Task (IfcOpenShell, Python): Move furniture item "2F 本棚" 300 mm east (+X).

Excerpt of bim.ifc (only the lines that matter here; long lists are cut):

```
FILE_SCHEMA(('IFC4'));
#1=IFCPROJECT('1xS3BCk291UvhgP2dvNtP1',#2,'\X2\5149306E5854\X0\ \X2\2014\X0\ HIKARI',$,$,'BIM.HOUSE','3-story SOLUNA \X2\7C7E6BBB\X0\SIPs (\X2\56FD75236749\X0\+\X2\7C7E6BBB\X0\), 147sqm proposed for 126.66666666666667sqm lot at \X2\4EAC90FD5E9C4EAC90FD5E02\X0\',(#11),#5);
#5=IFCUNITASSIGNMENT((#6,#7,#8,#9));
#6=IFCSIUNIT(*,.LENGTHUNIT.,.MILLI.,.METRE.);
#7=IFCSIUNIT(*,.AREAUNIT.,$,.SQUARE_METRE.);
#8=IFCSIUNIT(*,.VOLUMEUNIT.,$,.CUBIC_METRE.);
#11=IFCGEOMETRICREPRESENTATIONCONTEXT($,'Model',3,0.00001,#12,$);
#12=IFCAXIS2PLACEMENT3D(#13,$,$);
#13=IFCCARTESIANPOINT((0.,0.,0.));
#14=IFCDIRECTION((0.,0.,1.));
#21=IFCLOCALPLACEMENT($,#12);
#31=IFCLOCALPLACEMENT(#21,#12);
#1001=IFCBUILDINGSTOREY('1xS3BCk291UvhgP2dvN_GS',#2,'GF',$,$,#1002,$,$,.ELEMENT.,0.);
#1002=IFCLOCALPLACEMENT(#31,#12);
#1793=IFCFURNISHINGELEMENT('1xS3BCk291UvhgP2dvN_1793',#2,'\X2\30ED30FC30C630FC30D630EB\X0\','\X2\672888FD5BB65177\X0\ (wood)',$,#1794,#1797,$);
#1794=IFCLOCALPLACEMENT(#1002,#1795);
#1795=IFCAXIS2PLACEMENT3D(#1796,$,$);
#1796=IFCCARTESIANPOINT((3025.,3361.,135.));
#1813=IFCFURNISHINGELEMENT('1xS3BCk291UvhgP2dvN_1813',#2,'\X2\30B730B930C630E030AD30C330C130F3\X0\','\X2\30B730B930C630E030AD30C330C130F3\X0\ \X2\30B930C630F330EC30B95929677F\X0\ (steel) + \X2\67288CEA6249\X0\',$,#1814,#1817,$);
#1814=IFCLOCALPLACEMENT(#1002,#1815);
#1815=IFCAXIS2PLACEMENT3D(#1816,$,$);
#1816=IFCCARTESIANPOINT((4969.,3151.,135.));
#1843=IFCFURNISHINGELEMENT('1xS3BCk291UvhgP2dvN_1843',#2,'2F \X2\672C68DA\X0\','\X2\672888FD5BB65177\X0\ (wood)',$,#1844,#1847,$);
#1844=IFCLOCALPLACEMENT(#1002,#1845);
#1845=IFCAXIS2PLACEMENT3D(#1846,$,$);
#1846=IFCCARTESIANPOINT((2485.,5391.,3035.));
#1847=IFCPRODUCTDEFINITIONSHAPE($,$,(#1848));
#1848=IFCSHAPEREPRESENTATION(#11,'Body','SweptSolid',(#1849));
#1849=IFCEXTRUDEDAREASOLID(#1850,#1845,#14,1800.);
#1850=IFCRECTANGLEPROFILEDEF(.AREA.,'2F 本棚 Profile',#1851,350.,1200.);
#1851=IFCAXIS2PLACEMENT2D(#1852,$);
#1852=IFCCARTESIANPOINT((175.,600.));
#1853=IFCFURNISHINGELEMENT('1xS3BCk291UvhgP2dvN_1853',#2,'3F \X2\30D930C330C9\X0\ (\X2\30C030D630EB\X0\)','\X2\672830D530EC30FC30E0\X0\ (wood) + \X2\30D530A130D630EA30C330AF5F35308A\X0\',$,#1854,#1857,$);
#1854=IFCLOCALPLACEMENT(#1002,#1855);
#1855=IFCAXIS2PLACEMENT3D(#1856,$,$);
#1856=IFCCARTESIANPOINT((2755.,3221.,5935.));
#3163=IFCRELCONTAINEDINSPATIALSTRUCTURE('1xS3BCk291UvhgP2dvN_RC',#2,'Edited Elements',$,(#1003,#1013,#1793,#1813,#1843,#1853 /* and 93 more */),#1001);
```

```python
import ifcopenshell
import ifcopenshell.api.geometry
import ifcopenshell.util.placement
import ifcopenshell.util.unit

model = ifcopenshell.open("bim.ifc")
unit_scale = ifcopenshell.util.unit.calculate_unit_scale(model)

item = model.by_guid("1xS3BCk291UvhgP2dvN_1843")
matrix = ifcopenshell.util.placement.get_local_placement(item.ObjectPlacement)
matrix[0, 3] += 0.3 / unit_scale
ifcopenshell.api.geometry.edit_object_placement(model, product=item, matrix=matrix, is_si=False)

print(ifcopenshell.util.placement.get_local_placement(item.ObjectPlacement).round(3) + 0.0)

model.write("bim_rev.ifc")
```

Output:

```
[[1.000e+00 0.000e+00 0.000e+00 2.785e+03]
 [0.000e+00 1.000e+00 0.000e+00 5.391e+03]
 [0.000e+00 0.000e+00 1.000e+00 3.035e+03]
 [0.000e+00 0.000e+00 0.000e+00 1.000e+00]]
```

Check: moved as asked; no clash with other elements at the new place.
